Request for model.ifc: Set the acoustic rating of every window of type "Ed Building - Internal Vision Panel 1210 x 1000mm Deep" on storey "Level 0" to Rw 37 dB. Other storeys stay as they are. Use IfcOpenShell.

First a look at what the model holds.

```python
import ifcopenshell
import ifcopenshell.util.element

model = ifcopenshell.open("model.ifc")
print(model.schema)
storey = next(s for s in model.by_type("IfcBuildingStorey") if s.Name == "Level 0")
windows = [e for e in ifcopenshell.util.element.get_decomposition(storey) if e.is_a("IfcWindow")]
seen = {}
for e in windows:
    element_type = ifcopenshell.util.element.get_type(e)
    key = (element_type.Name if element_type != e and element_type else None, ifcopenshell.util.element.get_pset(e, "Pset_WindowCommon", "AcousticRating"))
    seen[key] = seen.get(key, 0) + 1
for (name, value), count in sorted(seen.items(), key=str):
    print(count, "x", name, "|", value)
```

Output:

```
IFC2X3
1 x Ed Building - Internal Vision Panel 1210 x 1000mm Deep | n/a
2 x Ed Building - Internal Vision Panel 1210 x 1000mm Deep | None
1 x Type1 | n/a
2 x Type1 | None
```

```python
import ifcopenshell
import ifcopenshell.api.pset
import ifcopenshell.util.element

model = ifcopenshell.open("model.ifc")

storey = next(s for s in model.by_type("IfcBuildingStorey") if s.Name == "Level 0")
windows = [e for e in ifcopenshell.util.element.get_decomposition(storey) if e.is_a("IfcWindow")]

count = 0
for e in windows:
    element_type = ifcopenshell.util.element.get_type(e)
    if element_type in (None, e) or element_type.Name != "Ed Building - Internal Vision Panel 1210 x 1000mm Deep":
        continue
    # add_pset returns the element's existing set when there is one.
    pset = ifcopenshell.api.pset.add_pset(model, product=e, name="Pset_WindowCommon")
    ifcopenshell.api.pset.edit_pset(model, pset=pset, properties={"AcousticRating": "Rw 37 dB"})
    count += 1

print(count, "windows updated")

model.write("model_v2.ifc")
```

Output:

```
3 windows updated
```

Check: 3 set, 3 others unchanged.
